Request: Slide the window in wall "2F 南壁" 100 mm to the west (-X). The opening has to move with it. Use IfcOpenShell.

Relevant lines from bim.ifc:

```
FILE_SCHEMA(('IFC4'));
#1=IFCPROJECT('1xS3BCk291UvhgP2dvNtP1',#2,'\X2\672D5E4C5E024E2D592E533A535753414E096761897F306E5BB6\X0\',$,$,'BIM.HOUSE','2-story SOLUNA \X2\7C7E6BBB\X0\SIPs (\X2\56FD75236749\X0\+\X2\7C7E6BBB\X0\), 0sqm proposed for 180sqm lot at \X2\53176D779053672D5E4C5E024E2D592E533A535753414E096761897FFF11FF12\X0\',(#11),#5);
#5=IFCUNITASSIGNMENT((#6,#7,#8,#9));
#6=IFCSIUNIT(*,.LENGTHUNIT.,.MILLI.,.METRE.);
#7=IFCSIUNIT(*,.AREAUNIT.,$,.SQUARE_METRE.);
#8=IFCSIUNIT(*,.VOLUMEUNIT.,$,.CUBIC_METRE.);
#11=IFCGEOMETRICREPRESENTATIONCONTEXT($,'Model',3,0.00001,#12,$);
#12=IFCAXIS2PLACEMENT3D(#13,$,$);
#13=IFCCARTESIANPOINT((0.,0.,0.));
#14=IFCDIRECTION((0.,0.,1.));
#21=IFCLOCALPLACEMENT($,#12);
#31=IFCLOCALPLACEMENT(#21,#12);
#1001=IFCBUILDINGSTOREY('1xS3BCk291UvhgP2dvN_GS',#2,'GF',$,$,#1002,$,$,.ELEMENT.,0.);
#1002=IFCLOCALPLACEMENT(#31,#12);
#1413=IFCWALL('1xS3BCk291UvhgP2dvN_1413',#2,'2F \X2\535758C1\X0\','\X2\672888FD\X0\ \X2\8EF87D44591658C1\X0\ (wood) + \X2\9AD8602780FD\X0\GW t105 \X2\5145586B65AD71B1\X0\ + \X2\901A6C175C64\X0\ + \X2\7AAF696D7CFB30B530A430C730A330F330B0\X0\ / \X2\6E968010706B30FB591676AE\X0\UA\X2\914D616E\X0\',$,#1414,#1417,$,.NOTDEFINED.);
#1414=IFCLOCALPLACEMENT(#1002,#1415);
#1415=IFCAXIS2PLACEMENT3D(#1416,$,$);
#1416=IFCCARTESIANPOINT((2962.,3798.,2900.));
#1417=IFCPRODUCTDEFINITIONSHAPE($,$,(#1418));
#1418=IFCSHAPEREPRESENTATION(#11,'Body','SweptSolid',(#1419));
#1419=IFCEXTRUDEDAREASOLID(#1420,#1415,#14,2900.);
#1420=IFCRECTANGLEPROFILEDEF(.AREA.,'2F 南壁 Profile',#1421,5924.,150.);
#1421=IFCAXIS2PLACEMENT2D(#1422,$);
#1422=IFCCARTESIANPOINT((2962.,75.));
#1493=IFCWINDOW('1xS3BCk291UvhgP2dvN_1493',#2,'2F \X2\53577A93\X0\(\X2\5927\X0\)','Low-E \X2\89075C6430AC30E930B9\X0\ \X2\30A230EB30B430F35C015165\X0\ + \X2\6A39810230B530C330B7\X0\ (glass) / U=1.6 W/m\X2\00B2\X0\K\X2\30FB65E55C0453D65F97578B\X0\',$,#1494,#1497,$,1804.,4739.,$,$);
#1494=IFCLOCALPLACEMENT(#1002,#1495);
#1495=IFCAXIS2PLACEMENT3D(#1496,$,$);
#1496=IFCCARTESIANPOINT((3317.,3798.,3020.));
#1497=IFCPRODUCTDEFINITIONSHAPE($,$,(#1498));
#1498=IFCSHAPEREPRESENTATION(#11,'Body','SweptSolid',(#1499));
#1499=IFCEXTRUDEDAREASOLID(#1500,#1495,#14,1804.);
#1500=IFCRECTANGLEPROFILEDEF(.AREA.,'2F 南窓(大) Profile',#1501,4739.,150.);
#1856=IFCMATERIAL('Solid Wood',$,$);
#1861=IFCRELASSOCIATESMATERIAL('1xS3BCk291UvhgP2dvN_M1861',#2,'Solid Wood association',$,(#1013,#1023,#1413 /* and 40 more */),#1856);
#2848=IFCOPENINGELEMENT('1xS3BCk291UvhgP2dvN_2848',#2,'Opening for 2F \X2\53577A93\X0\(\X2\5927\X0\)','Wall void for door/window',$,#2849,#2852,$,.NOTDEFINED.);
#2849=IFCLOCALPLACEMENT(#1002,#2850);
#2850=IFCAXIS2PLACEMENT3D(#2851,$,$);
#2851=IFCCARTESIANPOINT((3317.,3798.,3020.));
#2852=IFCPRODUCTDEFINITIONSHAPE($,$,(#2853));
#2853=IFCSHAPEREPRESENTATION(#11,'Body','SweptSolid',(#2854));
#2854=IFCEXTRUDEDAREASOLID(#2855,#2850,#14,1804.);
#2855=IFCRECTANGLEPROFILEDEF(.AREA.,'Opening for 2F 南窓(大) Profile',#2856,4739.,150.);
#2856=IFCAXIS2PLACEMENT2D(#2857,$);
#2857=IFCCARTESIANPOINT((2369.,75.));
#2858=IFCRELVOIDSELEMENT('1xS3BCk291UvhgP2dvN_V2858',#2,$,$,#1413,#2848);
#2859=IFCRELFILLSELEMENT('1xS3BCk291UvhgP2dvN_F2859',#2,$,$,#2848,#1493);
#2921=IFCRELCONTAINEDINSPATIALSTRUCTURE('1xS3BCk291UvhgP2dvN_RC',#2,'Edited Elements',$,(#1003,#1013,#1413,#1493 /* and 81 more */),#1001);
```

```python
import ifcopenshell
import ifcopenshell.api.geometry
import ifcopenshell.util.placement
import ifcopenshell.util.unit

model = ifcopenshell.open("bim.ifc")
unit_scale = ifcopenshell.util.unit.calculate_unit_scale(model)

window = model.by_guid("1xS3BCk291UvhgP2dvN_1493")
opening = window.FillsVoids[0].RelatingOpeningElement
wall = opening.VoidsElements[0].RelatingBuildingElement

wall_matrix = ifcopenshell.util.placement.get_local_placement(wall.ObjectPlacement)
shift = wall_matrix[:3, 0] * -0.1 / unit_scale
before = ifcopenshell.util.placement.get_local_placement(window.ObjectPlacement)[:3, 3].copy()

# The window is not placed relative to its opening, so move both.
for product in (opening, window):
    matrix = ifcopenshell.util.placement.get_local_placement(product.ObjectPlacement)
    matrix[:3, 3] += shift
    ifcopenshell.api.geometry.edit_object_placement(model, product=product, matrix=matrix, is_si=False)

after = ifcopenshell.util.placement.get_local_placement(window.ObjectPlacement)[:3, 3]
print("window moved by", (after - before).round(3) + 0.0)

model.write("bim_updated.ifc")
```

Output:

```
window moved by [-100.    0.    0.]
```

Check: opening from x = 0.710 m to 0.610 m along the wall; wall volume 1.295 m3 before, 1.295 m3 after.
